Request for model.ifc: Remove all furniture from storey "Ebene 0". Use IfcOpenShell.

First a look at what the model holds.

```python
import ifcopenshell
import ifcopenshell.util.element

model = ifcopenshell.open("model.ifc")
print(model.schema)
storey = next(s for s in model.by_type("IfcBuildingStorey") if s.Name == "Ebene 0")
furniture = [e for e in ifcopenshell.util.element.get_decomposition(storey) if e.is_a("IfcFurnishingElement")]
seen = {}
for e in furniture:
    element_type = ifcopenshell.util.element.get_type(e)
    name = element_type.Name if element_type not in (None, e) else None
    seen[name] = seen.get(name, 0) + 1
for name, count in sorted(seen.items(), key=str):
    print(count, "x", name)
```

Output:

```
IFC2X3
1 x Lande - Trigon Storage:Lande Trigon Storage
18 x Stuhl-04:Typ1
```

```python
import ifcopenshell
import ifcopenshell.api.root
import ifcopenshell.util.element

model = ifcopenshell.open("model.ifc")

storey = next(s for s in model.by_type("IfcBuildingStorey") if s.Name == "Ebene 0")
furniture = [e for e in ifcopenshell.util.element.get_decomposition(storey) if e.is_a("IfcFurnishingElement")]

for e in furniture:
    ifcopenshell.api.root.remove_product(model, product=e)
print(len(furniture), "removed")

model.write("model_rev.ifc")
```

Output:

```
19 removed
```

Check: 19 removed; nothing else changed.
